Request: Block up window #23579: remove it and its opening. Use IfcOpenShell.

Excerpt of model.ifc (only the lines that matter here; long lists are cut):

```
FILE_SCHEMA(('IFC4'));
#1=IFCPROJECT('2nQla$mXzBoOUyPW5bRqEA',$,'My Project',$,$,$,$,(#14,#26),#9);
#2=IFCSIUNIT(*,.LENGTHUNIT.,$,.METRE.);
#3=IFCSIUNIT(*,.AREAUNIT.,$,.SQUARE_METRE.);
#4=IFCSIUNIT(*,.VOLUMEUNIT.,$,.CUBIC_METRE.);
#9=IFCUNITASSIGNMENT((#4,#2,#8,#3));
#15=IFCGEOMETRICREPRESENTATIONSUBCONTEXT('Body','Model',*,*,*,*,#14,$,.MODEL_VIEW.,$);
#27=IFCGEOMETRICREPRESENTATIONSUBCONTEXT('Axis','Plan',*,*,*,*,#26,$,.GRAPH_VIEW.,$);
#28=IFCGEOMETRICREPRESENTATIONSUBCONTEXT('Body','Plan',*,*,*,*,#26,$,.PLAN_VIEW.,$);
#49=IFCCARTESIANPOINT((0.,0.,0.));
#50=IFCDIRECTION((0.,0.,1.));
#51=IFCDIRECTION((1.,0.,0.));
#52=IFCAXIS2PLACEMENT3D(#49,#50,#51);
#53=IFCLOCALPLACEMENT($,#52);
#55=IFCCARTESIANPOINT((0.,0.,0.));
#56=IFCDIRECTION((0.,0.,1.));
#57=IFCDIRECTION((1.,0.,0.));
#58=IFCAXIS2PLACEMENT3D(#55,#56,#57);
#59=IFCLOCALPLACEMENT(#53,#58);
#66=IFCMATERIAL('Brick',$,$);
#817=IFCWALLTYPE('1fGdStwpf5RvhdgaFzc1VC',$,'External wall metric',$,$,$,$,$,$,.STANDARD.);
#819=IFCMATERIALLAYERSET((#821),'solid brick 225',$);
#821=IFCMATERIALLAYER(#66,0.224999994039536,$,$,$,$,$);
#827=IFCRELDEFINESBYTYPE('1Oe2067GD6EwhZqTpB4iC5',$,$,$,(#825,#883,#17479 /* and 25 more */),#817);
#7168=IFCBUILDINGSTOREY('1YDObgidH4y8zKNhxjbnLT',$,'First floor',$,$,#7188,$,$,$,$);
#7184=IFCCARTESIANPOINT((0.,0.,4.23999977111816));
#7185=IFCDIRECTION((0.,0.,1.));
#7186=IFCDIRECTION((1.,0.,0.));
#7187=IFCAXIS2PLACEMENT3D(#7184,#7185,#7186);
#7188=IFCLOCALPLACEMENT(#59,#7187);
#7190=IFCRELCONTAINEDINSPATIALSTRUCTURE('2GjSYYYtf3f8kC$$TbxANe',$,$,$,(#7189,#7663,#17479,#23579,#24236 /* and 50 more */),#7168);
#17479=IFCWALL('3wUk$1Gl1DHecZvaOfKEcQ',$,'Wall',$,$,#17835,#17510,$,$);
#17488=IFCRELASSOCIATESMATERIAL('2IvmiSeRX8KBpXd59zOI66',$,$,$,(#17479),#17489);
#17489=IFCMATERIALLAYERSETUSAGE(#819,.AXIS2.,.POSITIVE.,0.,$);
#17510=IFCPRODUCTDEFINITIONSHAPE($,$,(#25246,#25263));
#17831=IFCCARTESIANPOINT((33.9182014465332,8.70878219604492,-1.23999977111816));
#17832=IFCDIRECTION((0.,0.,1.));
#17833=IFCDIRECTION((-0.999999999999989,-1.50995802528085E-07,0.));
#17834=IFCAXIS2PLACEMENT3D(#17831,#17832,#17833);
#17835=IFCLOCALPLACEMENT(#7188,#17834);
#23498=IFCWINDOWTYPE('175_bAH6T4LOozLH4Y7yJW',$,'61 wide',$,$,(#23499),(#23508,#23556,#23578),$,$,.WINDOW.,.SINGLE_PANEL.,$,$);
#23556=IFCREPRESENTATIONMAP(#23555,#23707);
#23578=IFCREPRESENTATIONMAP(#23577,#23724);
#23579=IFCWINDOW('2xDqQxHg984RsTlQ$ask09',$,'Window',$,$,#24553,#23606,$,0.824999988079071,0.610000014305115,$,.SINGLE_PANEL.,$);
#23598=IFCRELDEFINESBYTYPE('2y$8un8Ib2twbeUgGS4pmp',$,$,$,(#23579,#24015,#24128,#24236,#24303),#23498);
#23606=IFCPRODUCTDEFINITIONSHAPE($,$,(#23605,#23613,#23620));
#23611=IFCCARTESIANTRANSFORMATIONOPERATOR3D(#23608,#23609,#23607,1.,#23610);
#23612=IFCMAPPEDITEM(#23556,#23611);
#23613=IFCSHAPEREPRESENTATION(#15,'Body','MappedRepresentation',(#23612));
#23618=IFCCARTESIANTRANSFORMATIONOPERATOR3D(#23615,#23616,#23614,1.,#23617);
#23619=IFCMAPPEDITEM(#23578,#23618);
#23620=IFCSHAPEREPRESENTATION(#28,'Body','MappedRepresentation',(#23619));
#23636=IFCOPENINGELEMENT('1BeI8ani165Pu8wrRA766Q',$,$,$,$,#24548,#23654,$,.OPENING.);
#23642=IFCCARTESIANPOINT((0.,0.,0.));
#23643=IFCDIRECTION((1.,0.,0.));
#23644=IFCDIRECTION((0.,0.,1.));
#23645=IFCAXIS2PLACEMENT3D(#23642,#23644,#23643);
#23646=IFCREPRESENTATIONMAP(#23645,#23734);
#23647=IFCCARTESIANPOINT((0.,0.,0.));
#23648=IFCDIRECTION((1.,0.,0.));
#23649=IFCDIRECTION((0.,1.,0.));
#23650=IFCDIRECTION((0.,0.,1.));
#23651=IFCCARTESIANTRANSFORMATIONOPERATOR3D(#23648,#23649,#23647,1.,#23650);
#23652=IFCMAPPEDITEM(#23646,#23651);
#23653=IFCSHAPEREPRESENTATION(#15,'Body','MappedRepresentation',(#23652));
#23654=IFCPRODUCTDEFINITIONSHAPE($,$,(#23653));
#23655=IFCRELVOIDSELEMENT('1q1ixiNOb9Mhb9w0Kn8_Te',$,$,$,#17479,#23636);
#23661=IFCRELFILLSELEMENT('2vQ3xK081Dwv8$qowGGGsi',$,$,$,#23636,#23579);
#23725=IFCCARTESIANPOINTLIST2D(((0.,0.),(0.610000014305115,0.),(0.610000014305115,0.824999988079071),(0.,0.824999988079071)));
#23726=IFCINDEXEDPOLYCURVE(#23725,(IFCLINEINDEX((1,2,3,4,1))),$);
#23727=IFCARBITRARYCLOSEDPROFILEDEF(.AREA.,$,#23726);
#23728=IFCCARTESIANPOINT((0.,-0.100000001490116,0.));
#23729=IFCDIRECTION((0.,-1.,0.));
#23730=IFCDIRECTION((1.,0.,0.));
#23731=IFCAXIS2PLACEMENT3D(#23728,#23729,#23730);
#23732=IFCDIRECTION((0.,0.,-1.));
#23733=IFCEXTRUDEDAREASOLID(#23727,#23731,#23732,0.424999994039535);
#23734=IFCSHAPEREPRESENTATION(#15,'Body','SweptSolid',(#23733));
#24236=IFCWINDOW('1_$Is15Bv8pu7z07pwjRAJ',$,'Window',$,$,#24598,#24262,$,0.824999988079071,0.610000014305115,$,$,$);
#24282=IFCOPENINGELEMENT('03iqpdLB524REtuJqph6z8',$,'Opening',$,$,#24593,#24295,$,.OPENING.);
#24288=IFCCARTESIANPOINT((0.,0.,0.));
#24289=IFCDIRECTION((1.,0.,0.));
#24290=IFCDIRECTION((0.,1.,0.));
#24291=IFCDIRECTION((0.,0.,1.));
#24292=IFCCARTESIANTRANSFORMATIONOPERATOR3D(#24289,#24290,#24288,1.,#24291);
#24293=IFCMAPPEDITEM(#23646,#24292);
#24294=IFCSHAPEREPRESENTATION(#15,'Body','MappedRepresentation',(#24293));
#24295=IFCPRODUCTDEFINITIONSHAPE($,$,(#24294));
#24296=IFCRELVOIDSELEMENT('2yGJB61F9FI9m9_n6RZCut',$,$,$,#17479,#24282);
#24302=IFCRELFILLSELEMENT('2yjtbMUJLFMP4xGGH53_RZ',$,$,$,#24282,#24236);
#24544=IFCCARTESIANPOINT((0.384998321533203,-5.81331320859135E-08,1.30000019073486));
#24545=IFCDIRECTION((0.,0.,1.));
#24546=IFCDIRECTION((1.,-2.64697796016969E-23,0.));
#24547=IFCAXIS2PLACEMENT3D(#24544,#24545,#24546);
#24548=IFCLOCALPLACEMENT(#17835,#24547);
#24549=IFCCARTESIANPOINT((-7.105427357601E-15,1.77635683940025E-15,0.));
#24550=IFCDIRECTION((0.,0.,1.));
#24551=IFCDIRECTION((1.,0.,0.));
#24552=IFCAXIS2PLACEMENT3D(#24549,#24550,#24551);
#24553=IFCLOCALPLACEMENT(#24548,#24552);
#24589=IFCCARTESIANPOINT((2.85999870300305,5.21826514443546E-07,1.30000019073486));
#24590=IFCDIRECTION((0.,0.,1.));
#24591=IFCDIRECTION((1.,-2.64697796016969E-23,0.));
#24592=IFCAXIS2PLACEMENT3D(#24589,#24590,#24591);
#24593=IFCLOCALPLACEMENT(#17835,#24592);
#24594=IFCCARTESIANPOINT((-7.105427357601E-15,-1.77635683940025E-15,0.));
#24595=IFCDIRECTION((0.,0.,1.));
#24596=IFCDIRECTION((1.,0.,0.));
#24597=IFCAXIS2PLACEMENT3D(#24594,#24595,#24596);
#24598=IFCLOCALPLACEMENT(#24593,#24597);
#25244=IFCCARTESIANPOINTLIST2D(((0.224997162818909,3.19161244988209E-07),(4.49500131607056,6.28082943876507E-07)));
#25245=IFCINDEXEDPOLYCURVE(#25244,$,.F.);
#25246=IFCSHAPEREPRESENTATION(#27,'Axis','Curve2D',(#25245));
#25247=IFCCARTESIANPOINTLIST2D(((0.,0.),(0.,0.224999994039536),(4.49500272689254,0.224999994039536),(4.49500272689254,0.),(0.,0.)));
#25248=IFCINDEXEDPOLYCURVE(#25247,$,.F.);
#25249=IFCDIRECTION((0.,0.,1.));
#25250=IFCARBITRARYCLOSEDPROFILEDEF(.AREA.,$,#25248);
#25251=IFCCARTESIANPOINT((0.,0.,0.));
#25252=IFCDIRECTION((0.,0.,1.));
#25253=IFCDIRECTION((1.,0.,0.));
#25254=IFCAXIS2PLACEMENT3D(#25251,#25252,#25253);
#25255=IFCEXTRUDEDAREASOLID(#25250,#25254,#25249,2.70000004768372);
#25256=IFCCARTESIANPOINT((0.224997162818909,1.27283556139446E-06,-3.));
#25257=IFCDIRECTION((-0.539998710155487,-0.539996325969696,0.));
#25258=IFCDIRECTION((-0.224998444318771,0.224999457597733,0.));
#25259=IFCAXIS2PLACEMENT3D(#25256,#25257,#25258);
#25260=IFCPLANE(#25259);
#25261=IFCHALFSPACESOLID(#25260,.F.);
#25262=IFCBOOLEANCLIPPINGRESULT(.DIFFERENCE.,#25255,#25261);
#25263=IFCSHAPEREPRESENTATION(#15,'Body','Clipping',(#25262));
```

```python
import ifcopenshell
import ifcopenshell.api.feature
import ifcopenshell.api.root
import ifcopenshell.geom
import ifcopenshell.util.shape

model = ifcopenshell.open("model.ifc")
settings = ifcopenshell.geom.settings()


def volume(element):
    """Net volume in cubic metres, openings subtracted."""
    shape = ifcopenshell.geom.create_shape(settings, element)
    return ifcopenshell.util.shape.get_volume(shape.geometry)


window = model.by_guid("2xDqQxHg984RsTlQ$ask09")
opening = window.FillsVoids[0].RelatingOpeningElement
wall = opening.VoidsElements[0].RelatingBuildingElement
before = volume(wall)

ifcopenshell.api.root.remove_product(model, product=window)
ifcopenshell.api.feature.remove_feature(model, feature=opening)

after = volume(wall)

print(f"wall volume {before:.3f} -> {after:.3f} m3")

model.write("model_updated.ifc")
```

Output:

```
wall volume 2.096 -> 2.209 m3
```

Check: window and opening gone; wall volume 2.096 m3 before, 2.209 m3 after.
